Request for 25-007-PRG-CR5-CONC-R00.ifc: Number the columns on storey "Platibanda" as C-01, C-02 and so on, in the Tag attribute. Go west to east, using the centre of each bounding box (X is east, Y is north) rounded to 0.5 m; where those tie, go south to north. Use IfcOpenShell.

First a look at what the model holds.

```python
import ifcopenshell
import ifcopenshell.util.element
import ifcopenshell.util.placement

model = ifcopenshell.open("25-007-PRG-CR5-CONC-R00.ifc")
print(model.schema)
storey = next(s for s in model.by_type("IfcBuildingStorey") if s.Name == "Platibanda")
columns = [e for e in ifcopenshell.util.element.get_decomposition(storey) if e.is_a("IfcColumn")]
for e in sorted(columns, key=lambda e: e.id()):
    origin = ifcopenshell.util.placement.get_local_placement(e.ObjectPlacement)[:3, 3]
    print(e.id(), e.Tag, e.Name, origin.round(2) + 0.0, sep=" | ")
```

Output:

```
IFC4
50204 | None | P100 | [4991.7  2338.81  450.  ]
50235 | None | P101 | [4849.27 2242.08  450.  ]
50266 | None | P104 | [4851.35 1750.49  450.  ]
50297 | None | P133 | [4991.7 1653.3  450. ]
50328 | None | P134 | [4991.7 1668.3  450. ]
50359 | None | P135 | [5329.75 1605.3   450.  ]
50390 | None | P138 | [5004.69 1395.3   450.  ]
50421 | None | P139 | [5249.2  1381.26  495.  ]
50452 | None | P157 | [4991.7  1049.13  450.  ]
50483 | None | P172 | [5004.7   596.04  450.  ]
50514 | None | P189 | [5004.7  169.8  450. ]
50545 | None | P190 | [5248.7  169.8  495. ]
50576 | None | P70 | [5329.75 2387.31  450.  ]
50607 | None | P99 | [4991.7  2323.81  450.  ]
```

```python
import ifcopenshell
import ifcopenshell.geom
import ifcopenshell.util.element
import ifcopenshell.util.shape

model = ifcopenshell.open("25-007-PRG-CR5-CONC-R00.ifc")
settings = ifcopenshell.geom.settings()
settings.set("use-world-coords", True)


def centre(element):
    shape = ifcopenshell.geom.create_shape(settings, element)
    return ifcopenshell.util.shape.get_bbox_centroid(shape.geometry)


storey = next(s for s in model.by_type("IfcBuildingStorey") if s.Name == "Platibanda")
columns = [e for e in ifcopenshell.util.element.get_decomposition(storey) if e.is_a("IfcColumn")]

# Insertion points can sit at a corner or the storey origin, so sort by the geometry (in metres).
centres = {e: centre(e) for e in columns}
columns.sort(key=lambda e: (round(centres[e][0] / 0.5), centres[e][1]))

for i, e in enumerate(columns, start=1):
    number = f"C-{i:02d}"
    e.Tag = number
    print(e.id(), number)

model.write("25-007-PRG-CR5-CONC-R00_rev.ifc")
```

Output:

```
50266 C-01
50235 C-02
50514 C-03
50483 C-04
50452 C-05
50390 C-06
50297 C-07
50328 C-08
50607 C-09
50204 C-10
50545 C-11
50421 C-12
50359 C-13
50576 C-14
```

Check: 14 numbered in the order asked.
